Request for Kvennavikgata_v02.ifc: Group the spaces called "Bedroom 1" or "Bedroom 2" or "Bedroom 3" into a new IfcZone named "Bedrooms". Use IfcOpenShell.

First a look at what the model holds.

```python
import ifcopenshell

model = ifcopenshell.open("Kvennavikgata_v02.ifc")
print(model.schema)
seen = {}
for space in model.by_type("IfcSpace"):
    seen[space.Name] = seen.get(space.Name, 0) + 1
for name, count in sorted(seen.items(), key=str):
    print(count, "x", name)
print("zones:", [z.Name for z in model.by_type("IfcZone")][:20])
```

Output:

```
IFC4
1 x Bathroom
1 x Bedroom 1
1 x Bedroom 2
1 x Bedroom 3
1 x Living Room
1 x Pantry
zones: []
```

```python
import ifcopenshell
import ifcopenshell.api.group
import ifcopenshell.api.root

model = ifcopenshell.open("Kvennavikgata_v02.ifc")

names = {"Bedroom 1", "Bedroom 2", "Bedroom 3"}
spaces = [s for s in model.by_type("IfcSpace") if s.Name in names]

zone = ifcopenshell.api.root.create_entity(model, ifc_class="IfcZone", name="Bedrooms")
ifcopenshell.api.group.assign_group(model, products=spaces, group=zone)
print(len(spaces), "spaces in", zone.Name)

model.write("Kvennavikgata_v02_edited.ifc")
```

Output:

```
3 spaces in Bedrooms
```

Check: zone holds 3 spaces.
